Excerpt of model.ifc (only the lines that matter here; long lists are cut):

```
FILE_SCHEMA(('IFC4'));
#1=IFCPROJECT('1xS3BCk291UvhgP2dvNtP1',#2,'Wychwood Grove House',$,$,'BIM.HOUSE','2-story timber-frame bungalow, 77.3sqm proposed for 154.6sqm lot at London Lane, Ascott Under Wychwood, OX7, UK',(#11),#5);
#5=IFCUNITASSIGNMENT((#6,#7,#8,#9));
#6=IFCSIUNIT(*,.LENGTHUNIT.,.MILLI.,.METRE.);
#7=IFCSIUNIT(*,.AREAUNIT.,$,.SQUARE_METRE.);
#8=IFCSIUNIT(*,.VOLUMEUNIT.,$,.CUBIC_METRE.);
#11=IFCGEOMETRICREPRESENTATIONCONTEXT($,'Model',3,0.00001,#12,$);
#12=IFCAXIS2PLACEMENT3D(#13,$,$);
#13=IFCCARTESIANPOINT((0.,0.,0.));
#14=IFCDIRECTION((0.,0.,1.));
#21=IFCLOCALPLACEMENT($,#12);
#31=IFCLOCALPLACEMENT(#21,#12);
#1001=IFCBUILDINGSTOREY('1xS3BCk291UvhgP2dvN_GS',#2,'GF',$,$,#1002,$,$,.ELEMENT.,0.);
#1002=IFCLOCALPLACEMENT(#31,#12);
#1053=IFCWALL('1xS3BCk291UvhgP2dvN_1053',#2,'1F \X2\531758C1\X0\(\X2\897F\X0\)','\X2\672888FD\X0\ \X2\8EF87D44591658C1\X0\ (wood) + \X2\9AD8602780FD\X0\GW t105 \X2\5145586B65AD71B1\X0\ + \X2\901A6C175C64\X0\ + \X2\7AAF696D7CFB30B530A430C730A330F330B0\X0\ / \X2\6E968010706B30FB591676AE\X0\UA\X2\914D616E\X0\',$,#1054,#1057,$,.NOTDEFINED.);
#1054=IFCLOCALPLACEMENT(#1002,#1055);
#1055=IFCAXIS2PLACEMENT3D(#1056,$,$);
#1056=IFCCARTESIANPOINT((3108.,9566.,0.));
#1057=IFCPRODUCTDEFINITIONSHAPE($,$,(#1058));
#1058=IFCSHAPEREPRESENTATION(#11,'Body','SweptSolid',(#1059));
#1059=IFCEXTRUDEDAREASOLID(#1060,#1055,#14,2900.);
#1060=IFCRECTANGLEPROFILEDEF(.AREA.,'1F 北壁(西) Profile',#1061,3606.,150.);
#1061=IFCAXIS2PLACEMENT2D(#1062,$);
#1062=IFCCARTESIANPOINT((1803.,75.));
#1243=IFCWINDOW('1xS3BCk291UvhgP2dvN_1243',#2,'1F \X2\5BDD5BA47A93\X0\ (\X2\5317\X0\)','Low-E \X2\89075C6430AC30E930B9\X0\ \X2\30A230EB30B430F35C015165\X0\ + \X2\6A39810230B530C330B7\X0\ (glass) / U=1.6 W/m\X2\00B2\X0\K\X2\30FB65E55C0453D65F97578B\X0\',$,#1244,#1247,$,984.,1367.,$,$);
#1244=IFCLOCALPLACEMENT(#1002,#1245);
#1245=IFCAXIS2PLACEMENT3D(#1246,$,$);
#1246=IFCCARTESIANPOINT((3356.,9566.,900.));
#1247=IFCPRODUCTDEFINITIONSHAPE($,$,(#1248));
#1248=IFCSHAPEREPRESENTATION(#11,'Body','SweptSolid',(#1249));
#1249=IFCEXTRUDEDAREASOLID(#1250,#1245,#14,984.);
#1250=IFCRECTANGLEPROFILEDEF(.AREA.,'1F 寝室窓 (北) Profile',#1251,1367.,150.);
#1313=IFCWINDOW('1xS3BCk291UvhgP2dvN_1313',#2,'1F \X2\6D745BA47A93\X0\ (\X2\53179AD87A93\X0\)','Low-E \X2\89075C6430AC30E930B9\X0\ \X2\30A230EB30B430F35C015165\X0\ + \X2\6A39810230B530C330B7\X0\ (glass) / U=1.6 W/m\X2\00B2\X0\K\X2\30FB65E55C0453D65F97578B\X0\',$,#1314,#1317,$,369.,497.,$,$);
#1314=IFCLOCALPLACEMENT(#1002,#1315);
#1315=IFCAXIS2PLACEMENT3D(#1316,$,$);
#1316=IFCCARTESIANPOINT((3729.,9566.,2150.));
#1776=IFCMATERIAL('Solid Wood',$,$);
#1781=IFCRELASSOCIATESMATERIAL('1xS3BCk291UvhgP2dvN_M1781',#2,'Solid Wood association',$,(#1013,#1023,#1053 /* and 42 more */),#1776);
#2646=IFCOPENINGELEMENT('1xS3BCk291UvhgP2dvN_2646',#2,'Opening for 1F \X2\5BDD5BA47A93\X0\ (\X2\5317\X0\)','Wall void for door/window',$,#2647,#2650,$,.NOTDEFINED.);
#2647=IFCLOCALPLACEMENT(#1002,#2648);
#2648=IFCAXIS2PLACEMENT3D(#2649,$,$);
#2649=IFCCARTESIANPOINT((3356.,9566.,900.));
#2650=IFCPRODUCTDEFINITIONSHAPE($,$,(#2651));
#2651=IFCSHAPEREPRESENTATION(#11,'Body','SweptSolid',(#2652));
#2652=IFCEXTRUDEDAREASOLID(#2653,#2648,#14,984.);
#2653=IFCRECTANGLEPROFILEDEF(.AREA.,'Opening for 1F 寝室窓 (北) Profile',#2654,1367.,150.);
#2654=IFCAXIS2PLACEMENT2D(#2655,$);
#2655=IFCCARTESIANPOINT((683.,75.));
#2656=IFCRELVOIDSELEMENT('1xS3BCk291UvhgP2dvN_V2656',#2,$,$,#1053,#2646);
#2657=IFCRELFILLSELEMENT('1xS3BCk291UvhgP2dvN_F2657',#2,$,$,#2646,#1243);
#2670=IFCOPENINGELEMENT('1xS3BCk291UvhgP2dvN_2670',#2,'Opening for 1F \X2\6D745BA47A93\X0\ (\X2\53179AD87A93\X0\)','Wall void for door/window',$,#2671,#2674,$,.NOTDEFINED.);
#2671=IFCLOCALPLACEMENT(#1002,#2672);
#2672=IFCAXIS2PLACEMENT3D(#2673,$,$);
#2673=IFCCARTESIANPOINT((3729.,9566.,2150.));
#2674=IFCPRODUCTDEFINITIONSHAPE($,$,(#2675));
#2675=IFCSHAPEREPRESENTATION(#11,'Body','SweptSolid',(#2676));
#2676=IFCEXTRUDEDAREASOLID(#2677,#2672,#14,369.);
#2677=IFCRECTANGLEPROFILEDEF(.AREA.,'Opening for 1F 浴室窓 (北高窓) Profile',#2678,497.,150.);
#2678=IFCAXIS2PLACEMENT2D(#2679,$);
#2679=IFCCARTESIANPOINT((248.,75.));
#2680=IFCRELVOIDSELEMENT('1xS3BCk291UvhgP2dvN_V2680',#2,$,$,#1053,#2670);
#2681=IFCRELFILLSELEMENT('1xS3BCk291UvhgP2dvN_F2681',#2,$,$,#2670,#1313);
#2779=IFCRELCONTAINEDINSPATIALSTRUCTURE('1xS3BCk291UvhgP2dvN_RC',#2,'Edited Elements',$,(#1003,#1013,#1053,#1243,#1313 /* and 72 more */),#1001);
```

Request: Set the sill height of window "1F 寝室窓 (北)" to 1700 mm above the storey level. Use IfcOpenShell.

```python
import numpy as np
import ifcopenshell
import ifcopenshell.api.geometry
import ifcopenshell.geom
import ifcopenshell.util.element
import ifcopenshell.util.placement
import ifcopenshell.util.shape
import ifcopenshell.util.unit

model = ifcopenshell.open("model.ifc")
unit_scale = ifcopenshell.util.unit.calculate_unit_scale(model)

window = model.by_guid("1xS3BCk291UvhgP2dvN_1243")
opening = window.FillsVoids[0].RelatingOpeningElement
storey = ifcopenshell.util.element.get_container(window, ifc_class="IfcBuildingStorey")
level = ifcopenshell.util.placement.get_local_placement(storey.ObjectPlacement)[2, 3]

# The opening's origin need not be at the sill, so measure its lowest point.
shape = ifcopenshell.geom.create_shape(ifcopenshell.geom.settings(), opening)
bottom = ifcopenshell.util.shape.get_shape_bottom_elevation(shape, shape.geometry) / unit_scale
dz = level + 1.7 / unit_scale - bottom

shift = np.array([0.0, 0.0, dz])
# The window is not placed relative to its opening, so move both.
for product in (opening, window):
    matrix = ifcopenshell.util.placement.get_local_placement(product.ObjectPlacement)
    matrix[:3, 3] += shift
    ifcopenshell.api.geometry.edit_object_placement(model, product=product, matrix=matrix, is_si=False)

print(f"moved by {dz * unit_scale:+.3f} m")

model.write("model_updated.ifc")
```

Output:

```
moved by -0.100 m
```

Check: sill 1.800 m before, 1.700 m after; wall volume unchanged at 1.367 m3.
